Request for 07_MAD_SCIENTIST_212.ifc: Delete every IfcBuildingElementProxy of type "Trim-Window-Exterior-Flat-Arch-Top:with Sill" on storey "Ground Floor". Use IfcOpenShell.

First a look at what the model holds.

```python
import ifcopenshell
import ifcopenshell.util.element

model = ifcopenshell.open("07_MAD_SCIENTIST_212.ifc")
print(model.schema)
storey = next(s for s in model.by_type("IfcBuildingStorey") if s.Name == "Ground Floor")
proxies = [e for e in ifcopenshell.util.element.get_decomposition(storey) if e.is_a("IfcBuildingElementProxy")]
seen = {}
for e in proxies:
    element_type = ifcopenshell.util.element.get_type(e)
    name = element_type.Name if element_type not in (None, e) else None
    seen[name] = seen.get(name, 0) + 1
for name, count in sorted(seen.items(), key=str):
    print(count, "x", name)
```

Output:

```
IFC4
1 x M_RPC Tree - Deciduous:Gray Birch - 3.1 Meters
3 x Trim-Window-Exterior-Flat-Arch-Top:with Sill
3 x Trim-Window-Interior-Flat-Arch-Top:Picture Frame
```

```python
import ifcopenshell
import ifcopenshell.api.root
import ifcopenshell.util.element

model = ifcopenshell.open("07_MAD_SCIENTIST_212.ifc")

storey = next(s for s in model.by_type("IfcBuildingStorey") if s.Name == "Ground Floor")
proxies = [e for e in ifcopenshell.util.element.get_decomposition(storey) if e.is_a("IfcBuildingElementProxy")]
targets = [e for e in proxies if (t := ifcopenshell.util.element.get_type(e)) not in (None, e) and t.Name == "Trim-Window-Exterior-Flat-Arch-Top:with Sill"]

for e in targets:
    ifcopenshell.api.root.remove_product(model, product=e)
print(len(targets), "removed")

model.write("07_MAD_SCIENTIST_212_rev.ifc")
```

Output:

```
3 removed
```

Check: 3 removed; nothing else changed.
